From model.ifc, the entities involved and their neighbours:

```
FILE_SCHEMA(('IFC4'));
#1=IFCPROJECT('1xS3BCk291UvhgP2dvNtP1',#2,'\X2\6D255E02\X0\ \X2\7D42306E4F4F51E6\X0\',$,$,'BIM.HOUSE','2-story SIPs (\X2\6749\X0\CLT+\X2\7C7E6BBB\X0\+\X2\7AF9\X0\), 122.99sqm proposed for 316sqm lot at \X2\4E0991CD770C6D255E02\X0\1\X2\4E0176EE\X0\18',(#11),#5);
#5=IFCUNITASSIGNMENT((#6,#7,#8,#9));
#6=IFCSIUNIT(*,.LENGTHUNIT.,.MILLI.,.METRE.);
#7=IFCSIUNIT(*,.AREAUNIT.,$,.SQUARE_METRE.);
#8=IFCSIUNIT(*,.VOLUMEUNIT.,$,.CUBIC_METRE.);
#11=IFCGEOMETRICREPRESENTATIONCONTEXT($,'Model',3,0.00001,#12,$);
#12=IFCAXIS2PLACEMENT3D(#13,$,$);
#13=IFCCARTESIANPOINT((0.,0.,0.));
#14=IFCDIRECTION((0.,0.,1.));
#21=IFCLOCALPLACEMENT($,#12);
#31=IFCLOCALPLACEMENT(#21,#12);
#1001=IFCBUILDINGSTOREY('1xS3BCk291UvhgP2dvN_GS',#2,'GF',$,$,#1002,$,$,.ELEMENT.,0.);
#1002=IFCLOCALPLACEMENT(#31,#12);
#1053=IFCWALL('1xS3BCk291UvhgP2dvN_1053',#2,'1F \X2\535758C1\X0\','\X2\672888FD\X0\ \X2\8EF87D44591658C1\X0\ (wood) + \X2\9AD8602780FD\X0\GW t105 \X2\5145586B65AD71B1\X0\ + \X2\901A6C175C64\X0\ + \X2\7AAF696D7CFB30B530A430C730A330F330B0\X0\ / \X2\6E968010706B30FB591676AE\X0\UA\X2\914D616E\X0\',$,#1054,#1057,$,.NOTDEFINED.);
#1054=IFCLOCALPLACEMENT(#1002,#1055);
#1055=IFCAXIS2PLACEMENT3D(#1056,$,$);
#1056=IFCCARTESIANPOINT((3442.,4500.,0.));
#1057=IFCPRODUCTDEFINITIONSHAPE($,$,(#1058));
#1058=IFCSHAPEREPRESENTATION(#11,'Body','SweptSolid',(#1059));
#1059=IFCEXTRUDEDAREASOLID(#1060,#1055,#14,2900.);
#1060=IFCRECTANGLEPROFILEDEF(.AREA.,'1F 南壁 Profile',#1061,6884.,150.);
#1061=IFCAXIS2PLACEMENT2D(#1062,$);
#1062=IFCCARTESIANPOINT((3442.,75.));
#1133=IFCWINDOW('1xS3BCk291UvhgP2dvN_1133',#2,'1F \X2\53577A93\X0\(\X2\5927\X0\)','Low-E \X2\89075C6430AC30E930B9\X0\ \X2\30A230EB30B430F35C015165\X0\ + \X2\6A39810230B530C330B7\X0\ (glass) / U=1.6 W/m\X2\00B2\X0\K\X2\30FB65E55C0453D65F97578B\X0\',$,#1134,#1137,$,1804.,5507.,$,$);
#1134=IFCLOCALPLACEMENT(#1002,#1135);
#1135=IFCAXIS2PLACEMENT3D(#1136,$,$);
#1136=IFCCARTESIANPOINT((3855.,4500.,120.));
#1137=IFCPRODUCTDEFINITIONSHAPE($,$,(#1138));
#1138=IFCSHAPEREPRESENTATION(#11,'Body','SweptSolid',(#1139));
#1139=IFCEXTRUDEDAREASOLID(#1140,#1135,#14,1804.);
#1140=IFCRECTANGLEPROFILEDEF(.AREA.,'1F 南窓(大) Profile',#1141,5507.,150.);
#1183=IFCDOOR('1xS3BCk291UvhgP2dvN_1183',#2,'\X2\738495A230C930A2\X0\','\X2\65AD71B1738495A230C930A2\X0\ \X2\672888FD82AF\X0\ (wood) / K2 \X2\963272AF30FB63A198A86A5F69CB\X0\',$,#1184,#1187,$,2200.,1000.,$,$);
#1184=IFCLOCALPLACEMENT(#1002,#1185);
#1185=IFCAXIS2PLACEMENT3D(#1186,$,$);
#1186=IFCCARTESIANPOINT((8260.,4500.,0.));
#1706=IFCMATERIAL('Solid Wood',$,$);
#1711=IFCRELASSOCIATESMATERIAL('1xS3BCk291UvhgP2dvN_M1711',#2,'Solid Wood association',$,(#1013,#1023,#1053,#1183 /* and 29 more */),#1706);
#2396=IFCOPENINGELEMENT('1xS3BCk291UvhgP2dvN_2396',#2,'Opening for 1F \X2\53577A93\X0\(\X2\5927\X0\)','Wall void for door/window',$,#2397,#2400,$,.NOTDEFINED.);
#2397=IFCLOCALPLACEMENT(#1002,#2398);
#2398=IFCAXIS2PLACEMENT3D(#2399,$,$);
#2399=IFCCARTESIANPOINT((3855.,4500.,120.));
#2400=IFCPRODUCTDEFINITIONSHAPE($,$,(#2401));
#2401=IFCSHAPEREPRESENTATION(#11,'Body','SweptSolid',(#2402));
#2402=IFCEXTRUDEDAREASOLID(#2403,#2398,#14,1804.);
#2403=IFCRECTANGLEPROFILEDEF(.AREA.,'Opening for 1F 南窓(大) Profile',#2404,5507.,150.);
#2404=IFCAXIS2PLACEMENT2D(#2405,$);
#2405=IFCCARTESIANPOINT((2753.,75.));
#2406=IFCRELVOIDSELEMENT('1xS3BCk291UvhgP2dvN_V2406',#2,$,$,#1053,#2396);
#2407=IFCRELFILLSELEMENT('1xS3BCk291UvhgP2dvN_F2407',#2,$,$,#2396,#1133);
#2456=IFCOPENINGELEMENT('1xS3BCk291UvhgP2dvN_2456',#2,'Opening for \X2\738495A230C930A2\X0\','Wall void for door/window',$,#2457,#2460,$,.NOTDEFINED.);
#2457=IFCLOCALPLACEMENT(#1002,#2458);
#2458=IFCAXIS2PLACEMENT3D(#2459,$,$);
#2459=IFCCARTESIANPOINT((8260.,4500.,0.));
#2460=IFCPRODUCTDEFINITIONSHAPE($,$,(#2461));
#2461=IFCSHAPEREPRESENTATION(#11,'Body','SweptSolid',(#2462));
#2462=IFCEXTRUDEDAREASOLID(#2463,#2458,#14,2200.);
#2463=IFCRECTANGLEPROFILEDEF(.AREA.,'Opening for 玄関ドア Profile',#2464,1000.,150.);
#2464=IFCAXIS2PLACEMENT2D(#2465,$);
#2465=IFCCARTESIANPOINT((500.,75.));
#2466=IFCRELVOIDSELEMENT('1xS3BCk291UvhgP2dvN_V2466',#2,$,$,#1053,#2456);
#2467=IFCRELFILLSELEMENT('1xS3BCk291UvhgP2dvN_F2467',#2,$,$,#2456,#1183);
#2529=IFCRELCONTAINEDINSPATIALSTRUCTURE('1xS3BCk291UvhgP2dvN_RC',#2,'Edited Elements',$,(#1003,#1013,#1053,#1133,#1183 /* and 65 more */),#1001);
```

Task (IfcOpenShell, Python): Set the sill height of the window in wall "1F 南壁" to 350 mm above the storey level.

```python
import numpy as np
import ifcopenshell
import ifcopenshell.api.geometry
import ifcopenshell.geom
import ifcopenshell.util.element
import ifcopenshell.util.placement
import ifcopenshell.util.shape
import ifcopenshell.util.unit

model = ifcopenshell.open("model.ifc")
unit_scale = ifcopenshell.util.unit.calculate_unit_scale(model)

window = model.by_guid("1xS3BCk291UvhgP2dvN_1133")
opening = window.FillsVoids[0].RelatingOpeningElement
storey = ifcopenshell.util.element.get_container(window, ifc_class="IfcBuildingStorey")
level = ifcopenshell.util.placement.get_local_placement(storey.ObjectPlacement)[2, 3]

# The opening's origin need not be at the sill, so measure its lowest point.
shape = ifcopenshell.geom.create_shape(ifcopenshell.geom.settings(), opening)
bottom = ifcopenshell.util.shape.get_shape_bottom_elevation(shape, shape.geometry) / unit_scale
dz = level + 0.35 / unit_scale - bottom

shift = np.array([0.0, 0.0, dz])
# The window is not placed relative to its opening, so move both.
for product in (opening, window):
    matrix = ifcopenshell.util.placement.get_local_placement(product.ObjectPlacement)
    matrix[:3, 3] += shift
    ifcopenshell.api.geometry.edit_object_placement(model, product=product, matrix=matrix, is_si=False)

print(f"moved by {dz * unit_scale:+.3f} m")

model.write("model_updated.ifc")
```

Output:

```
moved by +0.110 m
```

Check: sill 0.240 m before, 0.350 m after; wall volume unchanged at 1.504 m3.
